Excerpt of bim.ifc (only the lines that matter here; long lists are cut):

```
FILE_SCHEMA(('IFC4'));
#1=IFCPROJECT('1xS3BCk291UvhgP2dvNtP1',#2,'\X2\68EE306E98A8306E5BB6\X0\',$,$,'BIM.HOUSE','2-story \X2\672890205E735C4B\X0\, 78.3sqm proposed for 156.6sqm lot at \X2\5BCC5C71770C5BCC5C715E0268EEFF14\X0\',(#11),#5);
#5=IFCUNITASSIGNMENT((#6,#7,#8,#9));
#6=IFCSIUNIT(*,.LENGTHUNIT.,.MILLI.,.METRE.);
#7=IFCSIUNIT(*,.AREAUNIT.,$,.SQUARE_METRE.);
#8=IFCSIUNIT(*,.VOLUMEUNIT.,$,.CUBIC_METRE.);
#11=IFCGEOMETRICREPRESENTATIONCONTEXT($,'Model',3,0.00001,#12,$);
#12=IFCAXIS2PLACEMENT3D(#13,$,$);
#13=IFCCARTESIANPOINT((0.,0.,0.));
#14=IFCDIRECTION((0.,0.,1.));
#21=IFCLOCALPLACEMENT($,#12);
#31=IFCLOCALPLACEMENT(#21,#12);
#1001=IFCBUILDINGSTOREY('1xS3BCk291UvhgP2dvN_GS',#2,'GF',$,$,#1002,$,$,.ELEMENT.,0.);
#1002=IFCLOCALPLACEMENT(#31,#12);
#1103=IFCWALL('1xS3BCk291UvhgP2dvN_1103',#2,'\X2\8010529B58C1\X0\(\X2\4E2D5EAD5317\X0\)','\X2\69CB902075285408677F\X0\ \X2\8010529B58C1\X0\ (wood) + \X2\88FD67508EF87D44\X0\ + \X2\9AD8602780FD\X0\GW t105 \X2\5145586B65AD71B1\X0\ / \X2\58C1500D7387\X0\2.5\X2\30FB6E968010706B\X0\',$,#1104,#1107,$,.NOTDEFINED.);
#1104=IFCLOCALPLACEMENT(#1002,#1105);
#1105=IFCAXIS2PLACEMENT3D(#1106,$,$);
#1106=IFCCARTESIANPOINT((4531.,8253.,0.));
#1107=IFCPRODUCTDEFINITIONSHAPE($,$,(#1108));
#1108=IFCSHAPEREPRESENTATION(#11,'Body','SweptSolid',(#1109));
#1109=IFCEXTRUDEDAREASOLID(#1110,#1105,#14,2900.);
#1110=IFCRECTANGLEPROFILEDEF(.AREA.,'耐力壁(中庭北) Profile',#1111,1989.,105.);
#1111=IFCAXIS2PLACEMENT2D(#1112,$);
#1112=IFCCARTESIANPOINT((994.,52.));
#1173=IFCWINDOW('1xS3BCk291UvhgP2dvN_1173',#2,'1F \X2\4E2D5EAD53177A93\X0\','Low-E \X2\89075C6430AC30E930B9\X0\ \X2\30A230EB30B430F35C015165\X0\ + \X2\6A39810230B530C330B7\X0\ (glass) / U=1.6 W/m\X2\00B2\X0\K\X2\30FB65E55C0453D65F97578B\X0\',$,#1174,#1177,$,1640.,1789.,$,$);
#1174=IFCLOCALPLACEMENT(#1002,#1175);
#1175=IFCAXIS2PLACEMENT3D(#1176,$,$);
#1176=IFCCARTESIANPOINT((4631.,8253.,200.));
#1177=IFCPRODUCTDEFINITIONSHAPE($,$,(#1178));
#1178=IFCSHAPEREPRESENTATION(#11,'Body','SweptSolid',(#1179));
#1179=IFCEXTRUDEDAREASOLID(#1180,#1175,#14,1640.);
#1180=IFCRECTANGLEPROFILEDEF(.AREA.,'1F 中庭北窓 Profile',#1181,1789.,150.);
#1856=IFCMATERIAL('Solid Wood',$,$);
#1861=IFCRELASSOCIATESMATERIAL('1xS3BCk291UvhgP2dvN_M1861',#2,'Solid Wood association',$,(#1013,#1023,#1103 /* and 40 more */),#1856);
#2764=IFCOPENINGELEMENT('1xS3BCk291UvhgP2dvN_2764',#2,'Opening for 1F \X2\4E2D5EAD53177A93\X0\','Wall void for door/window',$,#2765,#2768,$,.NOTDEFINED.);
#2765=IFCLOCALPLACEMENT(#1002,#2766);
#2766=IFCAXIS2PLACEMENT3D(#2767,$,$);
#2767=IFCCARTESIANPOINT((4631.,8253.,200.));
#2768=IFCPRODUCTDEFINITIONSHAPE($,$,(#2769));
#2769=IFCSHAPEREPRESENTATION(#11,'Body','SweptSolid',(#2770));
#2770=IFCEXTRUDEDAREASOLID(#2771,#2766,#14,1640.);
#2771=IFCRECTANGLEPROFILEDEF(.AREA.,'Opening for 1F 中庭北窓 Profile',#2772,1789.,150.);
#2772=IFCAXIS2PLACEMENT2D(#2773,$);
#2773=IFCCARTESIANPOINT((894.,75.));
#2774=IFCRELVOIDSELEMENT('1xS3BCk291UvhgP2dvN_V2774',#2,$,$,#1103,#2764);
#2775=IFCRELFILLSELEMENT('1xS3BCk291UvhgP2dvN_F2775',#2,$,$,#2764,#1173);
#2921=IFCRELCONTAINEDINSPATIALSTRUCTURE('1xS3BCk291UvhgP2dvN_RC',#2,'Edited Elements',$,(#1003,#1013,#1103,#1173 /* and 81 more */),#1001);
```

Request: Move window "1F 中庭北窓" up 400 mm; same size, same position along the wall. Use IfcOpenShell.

```python
import numpy as np
import ifcopenshell
import ifcopenshell.api.geometry
import ifcopenshell.util.placement
import ifcopenshell.util.unit

model = ifcopenshell.open("bim.ifc")
unit_scale = ifcopenshell.util.unit.calculate_unit_scale(model)

window = model.by_guid("1xS3BCk291UvhgP2dvN_1173")
opening = window.FillsVoids[0].RelatingOpeningElement
dz = 0.4 / unit_scale

shift = np.array([0.0, 0.0, dz])
# The window is not placed relative to its opening, so move both.
for product in (opening, window):
    matrix = ifcopenshell.util.placement.get_local_placement(product.ObjectPlacement)
    matrix[:3, 3] += shift
    ifcopenshell.api.geometry.edit_object_placement(model, product=product, matrix=matrix, is_si=False)

print(f"moved by {dz * unit_scale:+.3f} m")

model.write("bim_updated.ifc")
```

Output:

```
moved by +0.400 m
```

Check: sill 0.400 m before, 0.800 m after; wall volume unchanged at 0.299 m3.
